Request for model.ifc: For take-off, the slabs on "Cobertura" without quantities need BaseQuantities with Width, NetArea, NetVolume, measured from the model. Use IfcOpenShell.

First a look at what the model holds.

```python
import ifcopenshell
import ifcopenshell.util.element
import ifcopenshell.util.unit

model = ifcopenshell.open("model.ifc")
print(model.schema)
for unit_type in ("LENGTHUNIT", "AREAUNIT", "VOLUMEUNIT"):
    print(unit_type, ifcopenshell.util.unit.calculate_unit_scale(model, unit_type))
storey = next(s for s in model.by_type("IfcBuildingStorey") if s.Name == "Cobertura")
slabs = [e for e in ifcopenshell.util.element.get_decomposition(storey) if e.is_a("IfcSlab")]
for e in sorted(slabs, key=lambda e: e.id()):
    print(e.id(), e.is_a(), e.Name, list(ifcopenshell.util.element.get_psets(e, qtos_only=True)), sep=" | ")
```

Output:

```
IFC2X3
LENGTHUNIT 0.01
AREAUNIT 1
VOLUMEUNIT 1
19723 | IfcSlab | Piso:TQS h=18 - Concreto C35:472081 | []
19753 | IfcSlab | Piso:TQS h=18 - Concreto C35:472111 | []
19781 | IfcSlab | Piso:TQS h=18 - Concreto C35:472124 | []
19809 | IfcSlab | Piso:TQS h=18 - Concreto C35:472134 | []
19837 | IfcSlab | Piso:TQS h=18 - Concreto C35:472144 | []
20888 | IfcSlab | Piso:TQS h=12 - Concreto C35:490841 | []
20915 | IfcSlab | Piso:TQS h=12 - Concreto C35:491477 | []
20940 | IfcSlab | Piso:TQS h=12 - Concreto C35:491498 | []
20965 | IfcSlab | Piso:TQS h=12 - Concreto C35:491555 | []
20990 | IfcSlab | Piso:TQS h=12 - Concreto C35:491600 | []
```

```python
import ifcopenshell
import ifcopenshell.api.pset
import ifcopenshell.geom
import ifcopenshell.util.element
import ifcopenshell.util.shape
import ifcopenshell.util.unit

model = ifcopenshell.open("model.ifc")
unit_scale = ifcopenshell.util.unit.calculate_unit_scale(model)
area_scale = ifcopenshell.util.unit.calculate_unit_scale(model, "AREAUNIT")
volume_scale = ifcopenshell.util.unit.calculate_unit_scale(model, "VOLUMEUNIT")
settings = ifcopenshell.geom.settings()

storey = next(s for s in model.by_type("IfcBuildingStorey") if s.Name == "Cobertura")
slabs = [e for e in ifcopenshell.util.element.get_decomposition(storey) if e.is_a("IfcSlab")]

for e in sorted(slabs, key=lambda e: e.id()):
    if ifcopenshell.util.element.get_psets(e, qtos_only=True, should_inherit=False):
        continue
    # Geometry comes back in metres, in the element's own axes.
    shape = ifcopenshell.geom.create_shape(settings, e)
    values = {
        "Width": ifcopenshell.util.shape.get_z(shape.geometry) / unit_scale,
        "NetArea": ifcopenshell.util.shape.get_footprint_area(shape.geometry) / area_scale,
        "NetVolume": ifcopenshell.util.shape.get_volume(shape.geometry) / volume_scale,
    }
    qto = ifcopenshell.api.pset.add_qto(model, product=e, name="BaseQuantities")
    ifcopenshell.api.pset.edit_qto(model, qto=qto, properties=values)
    print(e.id(), {k: round(v, 3) for k, v in values.items()})

model.write("model_edited.ifc")
```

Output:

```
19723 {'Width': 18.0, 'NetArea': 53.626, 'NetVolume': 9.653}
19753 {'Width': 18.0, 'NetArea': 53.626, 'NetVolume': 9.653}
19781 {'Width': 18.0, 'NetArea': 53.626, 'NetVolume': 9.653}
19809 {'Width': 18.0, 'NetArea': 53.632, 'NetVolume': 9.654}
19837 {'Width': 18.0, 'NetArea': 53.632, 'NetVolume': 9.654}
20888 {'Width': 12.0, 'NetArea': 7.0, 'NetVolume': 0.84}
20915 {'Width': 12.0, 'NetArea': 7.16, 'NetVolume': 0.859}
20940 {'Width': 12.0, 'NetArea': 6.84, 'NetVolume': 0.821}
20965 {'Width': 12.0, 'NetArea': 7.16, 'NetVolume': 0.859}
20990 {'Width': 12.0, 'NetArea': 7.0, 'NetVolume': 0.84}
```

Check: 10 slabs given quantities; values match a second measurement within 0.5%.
